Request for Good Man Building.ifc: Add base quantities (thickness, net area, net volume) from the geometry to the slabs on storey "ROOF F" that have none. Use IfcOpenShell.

First a look at what the model holds.

```python
import ifcopenshell
import ifcopenshell.util.element
import ifcopenshell.util.unit

model = ifcopenshell.open("Good Man Building.ifc")
print(model.schema)
for unit_type in ("LENGTHUNIT", "AREAUNIT", "VOLUMEUNIT"):
    print(unit_type, ifcopenshell.util.unit.calculate_unit_scale(model, unit_type))
storey = next(s for s in model.by_type("IfcBuildingStorey") if s.Name == "ROOF F")
slabs = [e for e in ifcopenshell.util.element.get_decomposition(storey) if e.is_a("IfcSlab")]
for e in sorted(slabs, key=lambda e: e.id()):
    print(e.id(), e.is_a(), e.Name, list(ifcopenshell.util.element.get_psets(e, qtos_only=True)), sep=" | ")
```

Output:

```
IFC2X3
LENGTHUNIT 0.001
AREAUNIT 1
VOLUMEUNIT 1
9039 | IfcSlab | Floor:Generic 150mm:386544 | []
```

```python
import ifcopenshell
import ifcopenshell.api.pset
import ifcopenshell.geom
import ifcopenshell.util.element
import ifcopenshell.util.shape
import ifcopenshell.util.unit

model = ifcopenshell.open("Good Man Building.ifc")
unit_scale = ifcopenshell.util.unit.calculate_unit_scale(model)
area_scale = ifcopenshell.util.unit.calculate_unit_scale(model, "AREAUNIT")
volume_scale = ifcopenshell.util.unit.calculate_unit_scale(model, "VOLUMEUNIT")
settings = ifcopenshell.geom.settings()

storey = next(s for s in model.by_type("IfcBuildingStorey") if s.Name == "ROOF F")
slabs = [e for e in ifcopenshell.util.element.get_decomposition(storey) if e.is_a("IfcSlab")]

for e in sorted(slabs, key=lambda e: e.id()):
    if ifcopenshell.util.element.get_psets(e, qtos_only=True, should_inherit=False):
        continue
    # Geometry comes back in metres, in the element's own axes.
    shape = ifcopenshell.geom.create_shape(settings, e)
    values = {
        "Width": ifcopenshell.util.shape.get_z(shape.geometry) / unit_scale,
        "NetArea": ifcopenshell.util.shape.get_footprint_area(shape.geometry) / area_scale,
        "NetVolume": ifcopenshell.util.shape.get_volume(shape.geometry) / volume_scale,
    }
    qto = ifcopenshell.api.pset.add_qto(model, product=e, name="BaseQuantities")
    ifcopenshell.api.pset.edit_qto(model, qto=qto, properties=values)
    print(e.id(), {k: round(v, 3) for k, v in values.items()})

model.write("Good Man Building-out.ifc")
```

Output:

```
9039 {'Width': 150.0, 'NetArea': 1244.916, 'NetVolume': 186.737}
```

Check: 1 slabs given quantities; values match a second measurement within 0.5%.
